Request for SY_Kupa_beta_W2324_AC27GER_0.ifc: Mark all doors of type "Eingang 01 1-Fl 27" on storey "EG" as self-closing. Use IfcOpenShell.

First a look at what the model holds.

```python
import ifcopenshell
import ifcopenshell.util.element

model = ifcopenshell.open("SY_Kupa_beta_W2324_AC27GER_0.ifc")
print(model.schema)
storey = next(s for s in model.by_type("IfcBuildingStorey") if s.Name == "EG")
doors = [e for e in ifcopenshell.util.element.get_decomposition(storey) if e.is_a("IfcDoor")]
seen = {}
for e in doors:
    element_type = ifcopenshell.util.element.get_type(e)
    key = (element_type.Name if element_type != e and element_type else None, ifcopenshell.util.element.get_pset(e, "Pset_DoorCommon", "SelfClosing"))
    seen[key] = seen.get(key, 0) + 1
for (name, value), count in sorted(seen.items(), key=str):
    print(count, "x", name, "|", value)
```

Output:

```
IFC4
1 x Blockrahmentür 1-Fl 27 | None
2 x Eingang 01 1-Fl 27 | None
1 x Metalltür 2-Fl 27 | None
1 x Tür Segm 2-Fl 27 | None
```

```python
import ifcopenshell
import ifcopenshell.api.pset
import ifcopenshell.util.element

model = ifcopenshell.open("SY_Kupa_beta_W2324_AC27GER_0.ifc")

storey = next(s for s in model.by_type("IfcBuildingStorey") if s.Name == "EG")
doors = [e for e in ifcopenshell.util.element.get_decomposition(storey) if e.is_a("IfcDoor")]

count = 0
for e in doors:
    element_type = ifcopenshell.util.element.get_type(e)
    if element_type in (None, e) or element_type.Name != "Eingang 01 1-Fl 27":
        continue
    # add_pset returns the element's existing set when there is one.
    pset = ifcopenshell.api.pset.add_pset(model, product=e, name="Pset_DoorCommon")
    ifcopenshell.api.pset.edit_pset(model, pset=pset, properties={"SelfClosing": True})
    count += 1

print(count, "doors updated")

model.write("SY_Kupa_beta_W2324_AC27GER_0_edited.ifc")
```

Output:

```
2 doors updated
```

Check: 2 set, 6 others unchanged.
